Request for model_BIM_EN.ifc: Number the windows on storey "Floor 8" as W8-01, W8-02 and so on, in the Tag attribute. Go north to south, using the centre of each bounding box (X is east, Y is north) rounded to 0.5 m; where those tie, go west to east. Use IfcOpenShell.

First a look at what the model holds.

```python
import ifcopenshell
import ifcopenshell.util.element
import ifcopenshell.util.placement

model = ifcopenshell.open("model_BIM_EN.ifc")
print(model.schema)
storey = next(s for s in model.by_type("IfcBuildingStorey") if s.Name == "Floor 8")
windows = [e for e in ifcopenshell.util.element.get_decomposition(storey) if e.is_a("IfcWindow")]
for e in sorted(windows, key=lambda e: e.id()):
    origin = ifcopenshell.util.placement.get_local_placement(e.ObjectPlacement)[:3, 3]
    print(e.id(), e.Tag, e.Name, origin.round(2) + 0.0, sep=" | ")
```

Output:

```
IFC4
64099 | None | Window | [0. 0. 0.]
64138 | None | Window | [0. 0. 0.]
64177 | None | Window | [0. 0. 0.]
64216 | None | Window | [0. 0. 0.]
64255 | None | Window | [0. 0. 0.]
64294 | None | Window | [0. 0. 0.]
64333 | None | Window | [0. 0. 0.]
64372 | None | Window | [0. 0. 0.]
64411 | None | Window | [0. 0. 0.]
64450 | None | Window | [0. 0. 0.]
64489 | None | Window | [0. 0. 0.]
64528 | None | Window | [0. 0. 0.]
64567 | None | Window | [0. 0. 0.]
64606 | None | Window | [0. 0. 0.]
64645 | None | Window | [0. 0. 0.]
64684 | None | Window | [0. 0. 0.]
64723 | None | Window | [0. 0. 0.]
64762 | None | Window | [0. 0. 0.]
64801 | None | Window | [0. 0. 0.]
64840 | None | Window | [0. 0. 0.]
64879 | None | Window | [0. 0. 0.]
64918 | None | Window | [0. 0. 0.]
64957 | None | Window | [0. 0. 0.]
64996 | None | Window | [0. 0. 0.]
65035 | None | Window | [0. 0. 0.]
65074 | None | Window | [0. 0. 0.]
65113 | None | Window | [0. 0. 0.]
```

```python
import ifcopenshell
import ifcopenshell.geom
import ifcopenshell.util.element
import ifcopenshell.util.shape

model = ifcopenshell.open("model_BIM_EN.ifc")
settings = ifcopenshell.geom.settings()
settings.set("use-world-coords", True)


def centre(element):
    shape = ifcopenshell.geom.create_shape(settings, element)
    return ifcopenshell.util.shape.get_bbox_centroid(shape.geometry)


storey = next(s for s in model.by_type("IfcBuildingStorey") if s.Name == "Floor 8")
windows = [e for e in ifcopenshell.util.element.get_decomposition(storey) if e.is_a("IfcWindow")]

# Insertion points can sit at a corner or the storey origin, so sort by the geometry (in metres).
centres = {e: centre(e) for e in windows}
windows.sort(key=lambda e: (-round(centres[e][1] / 0.5), centres[e][0]))

for i, e in enumerate(windows, start=1):
    number = f"W8-{i:02d}"
    e.Tag = number
    print(e.id(), number)

model.write("model_BIM_EN_rev.ifc")
```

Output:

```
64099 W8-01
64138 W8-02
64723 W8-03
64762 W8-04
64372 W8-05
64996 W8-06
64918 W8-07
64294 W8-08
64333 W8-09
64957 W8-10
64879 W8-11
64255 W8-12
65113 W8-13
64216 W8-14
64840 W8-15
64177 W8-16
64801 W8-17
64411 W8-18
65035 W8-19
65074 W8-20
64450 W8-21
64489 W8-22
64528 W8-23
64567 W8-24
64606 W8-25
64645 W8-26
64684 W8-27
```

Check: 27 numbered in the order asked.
